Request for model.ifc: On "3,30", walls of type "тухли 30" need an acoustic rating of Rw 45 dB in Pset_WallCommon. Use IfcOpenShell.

First a look at what the model holds.

```python
import ifcopenshell
import ifcopenshell.util.element

model = ifcopenshell.open("model.ifc")
print(model.schema)
storey = next(s for s in model.by_type("IfcBuildingStorey") if s.Name == "3,30")
walls = [e for e in ifcopenshell.util.element.get_decomposition(storey) if e.is_a("IfcWall")]
seen = {}
for e in walls:
    element_type = ifcopenshell.util.element.get_type(e)
    key = (element_type.Name if element_type != e and element_type else None, ifcopenshell.util.element.get_pset(e, "Pset_WallCommon", "AcousticRating"))
    seen[key] = seen.get(key, 0) + 1
for (name, value), count in sorted(seen.items(), key=str):
    print(count, "x", name, "|", value)
```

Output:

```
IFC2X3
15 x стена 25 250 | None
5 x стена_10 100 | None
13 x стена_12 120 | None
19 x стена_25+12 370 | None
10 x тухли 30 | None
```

```python
import ifcopenshell
import ifcopenshell.api.pset
import ifcopenshell.util.element

model = ifcopenshell.open("model.ifc")

storey = next(s for s in model.by_type("IfcBuildingStorey") if s.Name == "3,30")
walls = [e for e in ifcopenshell.util.element.get_decomposition(storey) if e.is_a("IfcWall")]

count = 0
for e in walls:
    element_type = ifcopenshell.util.element.get_type(e)
    if element_type in (None, e) or element_type.Name != "тухли 30":
        continue
    # add_pset returns the element's existing set when there is one.
    pset = ifcopenshell.api.pset.add_pset(model, product=e, name="Pset_WallCommon")
    ifcopenshell.api.pset.edit_pset(model, pset=pset, properties={"AcousticRating": "Rw 45 dB"})
    count += 1

print(count, "walls updated")

model.write("model_updated.ifc")
```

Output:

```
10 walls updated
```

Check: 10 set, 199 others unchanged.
